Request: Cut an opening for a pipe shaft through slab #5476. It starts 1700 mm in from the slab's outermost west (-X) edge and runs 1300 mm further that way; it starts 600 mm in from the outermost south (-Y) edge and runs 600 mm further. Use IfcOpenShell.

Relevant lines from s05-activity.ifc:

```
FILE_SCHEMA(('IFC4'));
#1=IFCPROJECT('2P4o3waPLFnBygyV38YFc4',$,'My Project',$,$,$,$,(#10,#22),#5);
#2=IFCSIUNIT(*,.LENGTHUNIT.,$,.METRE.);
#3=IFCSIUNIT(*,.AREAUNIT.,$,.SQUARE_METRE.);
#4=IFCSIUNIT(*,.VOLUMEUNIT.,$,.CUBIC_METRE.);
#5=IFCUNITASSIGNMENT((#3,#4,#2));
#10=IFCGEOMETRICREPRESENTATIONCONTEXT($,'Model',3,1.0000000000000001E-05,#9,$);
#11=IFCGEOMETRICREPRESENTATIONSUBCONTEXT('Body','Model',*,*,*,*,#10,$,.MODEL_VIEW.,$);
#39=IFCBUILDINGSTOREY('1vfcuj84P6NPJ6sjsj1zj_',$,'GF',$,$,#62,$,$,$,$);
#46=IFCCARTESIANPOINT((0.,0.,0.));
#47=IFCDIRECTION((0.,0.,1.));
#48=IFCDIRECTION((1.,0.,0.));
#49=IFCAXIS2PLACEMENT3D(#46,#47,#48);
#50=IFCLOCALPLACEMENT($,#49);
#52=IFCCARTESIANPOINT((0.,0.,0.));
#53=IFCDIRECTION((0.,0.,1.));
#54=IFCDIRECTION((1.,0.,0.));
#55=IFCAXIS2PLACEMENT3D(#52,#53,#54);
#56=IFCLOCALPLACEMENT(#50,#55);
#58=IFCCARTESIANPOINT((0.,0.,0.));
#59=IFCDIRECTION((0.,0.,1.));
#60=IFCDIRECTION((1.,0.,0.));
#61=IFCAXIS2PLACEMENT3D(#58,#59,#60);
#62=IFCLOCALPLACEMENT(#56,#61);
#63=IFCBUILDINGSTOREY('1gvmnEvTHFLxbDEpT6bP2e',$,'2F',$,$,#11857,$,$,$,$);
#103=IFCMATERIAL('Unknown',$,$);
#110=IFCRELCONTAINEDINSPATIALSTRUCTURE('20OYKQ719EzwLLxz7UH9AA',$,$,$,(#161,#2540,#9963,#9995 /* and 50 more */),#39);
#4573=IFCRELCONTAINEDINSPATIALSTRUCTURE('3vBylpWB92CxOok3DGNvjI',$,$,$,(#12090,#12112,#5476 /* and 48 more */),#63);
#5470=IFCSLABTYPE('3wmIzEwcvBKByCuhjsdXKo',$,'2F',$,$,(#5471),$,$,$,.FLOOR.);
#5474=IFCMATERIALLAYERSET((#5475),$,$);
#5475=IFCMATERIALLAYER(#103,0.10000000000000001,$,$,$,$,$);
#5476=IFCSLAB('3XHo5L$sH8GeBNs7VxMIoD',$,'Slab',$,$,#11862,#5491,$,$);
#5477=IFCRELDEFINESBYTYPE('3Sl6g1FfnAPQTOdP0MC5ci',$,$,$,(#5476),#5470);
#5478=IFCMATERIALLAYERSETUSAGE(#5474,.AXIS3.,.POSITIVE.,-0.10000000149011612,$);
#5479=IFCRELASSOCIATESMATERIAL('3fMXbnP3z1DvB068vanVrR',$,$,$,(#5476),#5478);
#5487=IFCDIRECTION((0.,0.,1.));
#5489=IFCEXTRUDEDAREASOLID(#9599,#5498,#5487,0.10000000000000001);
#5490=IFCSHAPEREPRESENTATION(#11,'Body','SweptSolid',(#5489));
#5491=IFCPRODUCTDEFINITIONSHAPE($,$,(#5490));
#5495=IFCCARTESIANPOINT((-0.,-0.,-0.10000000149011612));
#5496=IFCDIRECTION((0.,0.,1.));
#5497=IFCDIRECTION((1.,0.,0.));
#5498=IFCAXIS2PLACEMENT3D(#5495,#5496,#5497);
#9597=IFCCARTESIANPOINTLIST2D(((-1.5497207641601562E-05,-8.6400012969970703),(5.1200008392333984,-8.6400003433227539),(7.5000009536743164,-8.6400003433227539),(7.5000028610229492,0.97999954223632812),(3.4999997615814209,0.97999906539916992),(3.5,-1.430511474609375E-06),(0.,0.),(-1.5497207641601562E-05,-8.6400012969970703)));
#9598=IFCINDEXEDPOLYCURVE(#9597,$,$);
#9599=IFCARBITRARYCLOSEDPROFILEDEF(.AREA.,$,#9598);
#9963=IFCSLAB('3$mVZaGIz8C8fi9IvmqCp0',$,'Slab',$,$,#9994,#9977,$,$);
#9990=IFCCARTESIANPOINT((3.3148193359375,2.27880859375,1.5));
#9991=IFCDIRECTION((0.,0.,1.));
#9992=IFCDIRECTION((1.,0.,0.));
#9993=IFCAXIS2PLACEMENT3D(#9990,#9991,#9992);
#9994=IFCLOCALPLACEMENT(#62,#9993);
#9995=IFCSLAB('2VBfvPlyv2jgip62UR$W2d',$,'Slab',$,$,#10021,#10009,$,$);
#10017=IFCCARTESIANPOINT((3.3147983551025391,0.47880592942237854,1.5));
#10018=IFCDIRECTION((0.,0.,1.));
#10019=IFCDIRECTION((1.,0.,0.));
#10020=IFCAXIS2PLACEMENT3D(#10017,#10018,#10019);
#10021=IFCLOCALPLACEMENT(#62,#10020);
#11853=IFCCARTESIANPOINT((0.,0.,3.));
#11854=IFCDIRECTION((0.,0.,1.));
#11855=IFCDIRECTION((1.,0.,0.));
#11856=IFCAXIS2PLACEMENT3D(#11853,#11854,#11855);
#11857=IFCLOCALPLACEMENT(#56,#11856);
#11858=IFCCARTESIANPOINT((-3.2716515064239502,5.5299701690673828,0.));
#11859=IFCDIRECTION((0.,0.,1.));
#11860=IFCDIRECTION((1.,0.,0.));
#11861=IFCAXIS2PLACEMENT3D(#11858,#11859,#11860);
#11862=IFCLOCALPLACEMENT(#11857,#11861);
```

```python
import numpy as np
import ifcopenshell
import ifcopenshell.api.feature
import ifcopenshell.api.geometry
import ifcopenshell.api.root
import ifcopenshell.geom
import ifcopenshell.util.placement
import ifcopenshell.util.representation
import ifcopenshell.util.shape
import ifcopenshell.util.unit

model = ifcopenshell.open("s05-activity.ifc")
unit_scale = ifcopenshell.util.unit.calculate_unit_scale(model)
settings = ifcopenshell.geom.settings()


def volume(element):
    """Net volume in cubic metres, openings subtracted."""
    shape = ifcopenshell.geom.create_shape(settings, element)
    return ifcopenshell.util.shape.get_volume(shape.geometry)


slab = model.by_guid("3XHo5L$sH8GeBNs7VxMIoD")
before = volume(slab)

# Extent in the slab's own axes, in metres. The edges named are its -X and -Y sides.
slab_shape = ifcopenshell.geom.create_shape(settings, slab)
vertices = ifcopenshell.util.shape.get_vertices(slab_shape.geometry)
x_min, y_min, bottom = vertices.min(axis=0)
top = vertices[:, 2].max()

opening = ifcopenshell.api.root.create_entity(model, ifc_class="IfcOpeningElement", name="Pipe shaft opening", predefined_type="OPENING")
context = ifcopenshell.util.representation.get_context(model, "Model", "Body", "MODEL_VIEW")
width, depth = 1.3, 0.6
outline = [(0.0, 0.0), (width, 0.0), (width, depth), (0.0, depth), (0.0, 0.0)]
# Overshoot both faces by 50 mm so the cut is clean.
shape = ifcopenshell.api.geometry.add_slab_representation(
    model, context=context, depth=top - bottom + 0.1, polyline=outline
)
ifcopenshell.api.geometry.assign_representation(model, product=opening, representation=shape)

matrix = ifcopenshell.util.placement.get_local_placement(slab.ObjectPlacement)
matrix[:, 3] = matrix @ np.append(np.array([x_min + 1.7, y_min + 0.6, bottom - 0.05]) / unit_scale, 1.0)
ifcopenshell.api.geometry.edit_object_placement(model, product=opening, matrix=matrix, is_si=False)
ifcopenshell.api.feature.add_feature(model, feature=opening, element=slab)

after = volume(slab)

print(f"slab volume {before:.3f} -> {after:.3f} m3")

model.write("s05-activity_edited.ifc")
```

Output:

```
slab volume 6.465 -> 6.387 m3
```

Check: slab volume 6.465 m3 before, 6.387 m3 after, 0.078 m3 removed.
